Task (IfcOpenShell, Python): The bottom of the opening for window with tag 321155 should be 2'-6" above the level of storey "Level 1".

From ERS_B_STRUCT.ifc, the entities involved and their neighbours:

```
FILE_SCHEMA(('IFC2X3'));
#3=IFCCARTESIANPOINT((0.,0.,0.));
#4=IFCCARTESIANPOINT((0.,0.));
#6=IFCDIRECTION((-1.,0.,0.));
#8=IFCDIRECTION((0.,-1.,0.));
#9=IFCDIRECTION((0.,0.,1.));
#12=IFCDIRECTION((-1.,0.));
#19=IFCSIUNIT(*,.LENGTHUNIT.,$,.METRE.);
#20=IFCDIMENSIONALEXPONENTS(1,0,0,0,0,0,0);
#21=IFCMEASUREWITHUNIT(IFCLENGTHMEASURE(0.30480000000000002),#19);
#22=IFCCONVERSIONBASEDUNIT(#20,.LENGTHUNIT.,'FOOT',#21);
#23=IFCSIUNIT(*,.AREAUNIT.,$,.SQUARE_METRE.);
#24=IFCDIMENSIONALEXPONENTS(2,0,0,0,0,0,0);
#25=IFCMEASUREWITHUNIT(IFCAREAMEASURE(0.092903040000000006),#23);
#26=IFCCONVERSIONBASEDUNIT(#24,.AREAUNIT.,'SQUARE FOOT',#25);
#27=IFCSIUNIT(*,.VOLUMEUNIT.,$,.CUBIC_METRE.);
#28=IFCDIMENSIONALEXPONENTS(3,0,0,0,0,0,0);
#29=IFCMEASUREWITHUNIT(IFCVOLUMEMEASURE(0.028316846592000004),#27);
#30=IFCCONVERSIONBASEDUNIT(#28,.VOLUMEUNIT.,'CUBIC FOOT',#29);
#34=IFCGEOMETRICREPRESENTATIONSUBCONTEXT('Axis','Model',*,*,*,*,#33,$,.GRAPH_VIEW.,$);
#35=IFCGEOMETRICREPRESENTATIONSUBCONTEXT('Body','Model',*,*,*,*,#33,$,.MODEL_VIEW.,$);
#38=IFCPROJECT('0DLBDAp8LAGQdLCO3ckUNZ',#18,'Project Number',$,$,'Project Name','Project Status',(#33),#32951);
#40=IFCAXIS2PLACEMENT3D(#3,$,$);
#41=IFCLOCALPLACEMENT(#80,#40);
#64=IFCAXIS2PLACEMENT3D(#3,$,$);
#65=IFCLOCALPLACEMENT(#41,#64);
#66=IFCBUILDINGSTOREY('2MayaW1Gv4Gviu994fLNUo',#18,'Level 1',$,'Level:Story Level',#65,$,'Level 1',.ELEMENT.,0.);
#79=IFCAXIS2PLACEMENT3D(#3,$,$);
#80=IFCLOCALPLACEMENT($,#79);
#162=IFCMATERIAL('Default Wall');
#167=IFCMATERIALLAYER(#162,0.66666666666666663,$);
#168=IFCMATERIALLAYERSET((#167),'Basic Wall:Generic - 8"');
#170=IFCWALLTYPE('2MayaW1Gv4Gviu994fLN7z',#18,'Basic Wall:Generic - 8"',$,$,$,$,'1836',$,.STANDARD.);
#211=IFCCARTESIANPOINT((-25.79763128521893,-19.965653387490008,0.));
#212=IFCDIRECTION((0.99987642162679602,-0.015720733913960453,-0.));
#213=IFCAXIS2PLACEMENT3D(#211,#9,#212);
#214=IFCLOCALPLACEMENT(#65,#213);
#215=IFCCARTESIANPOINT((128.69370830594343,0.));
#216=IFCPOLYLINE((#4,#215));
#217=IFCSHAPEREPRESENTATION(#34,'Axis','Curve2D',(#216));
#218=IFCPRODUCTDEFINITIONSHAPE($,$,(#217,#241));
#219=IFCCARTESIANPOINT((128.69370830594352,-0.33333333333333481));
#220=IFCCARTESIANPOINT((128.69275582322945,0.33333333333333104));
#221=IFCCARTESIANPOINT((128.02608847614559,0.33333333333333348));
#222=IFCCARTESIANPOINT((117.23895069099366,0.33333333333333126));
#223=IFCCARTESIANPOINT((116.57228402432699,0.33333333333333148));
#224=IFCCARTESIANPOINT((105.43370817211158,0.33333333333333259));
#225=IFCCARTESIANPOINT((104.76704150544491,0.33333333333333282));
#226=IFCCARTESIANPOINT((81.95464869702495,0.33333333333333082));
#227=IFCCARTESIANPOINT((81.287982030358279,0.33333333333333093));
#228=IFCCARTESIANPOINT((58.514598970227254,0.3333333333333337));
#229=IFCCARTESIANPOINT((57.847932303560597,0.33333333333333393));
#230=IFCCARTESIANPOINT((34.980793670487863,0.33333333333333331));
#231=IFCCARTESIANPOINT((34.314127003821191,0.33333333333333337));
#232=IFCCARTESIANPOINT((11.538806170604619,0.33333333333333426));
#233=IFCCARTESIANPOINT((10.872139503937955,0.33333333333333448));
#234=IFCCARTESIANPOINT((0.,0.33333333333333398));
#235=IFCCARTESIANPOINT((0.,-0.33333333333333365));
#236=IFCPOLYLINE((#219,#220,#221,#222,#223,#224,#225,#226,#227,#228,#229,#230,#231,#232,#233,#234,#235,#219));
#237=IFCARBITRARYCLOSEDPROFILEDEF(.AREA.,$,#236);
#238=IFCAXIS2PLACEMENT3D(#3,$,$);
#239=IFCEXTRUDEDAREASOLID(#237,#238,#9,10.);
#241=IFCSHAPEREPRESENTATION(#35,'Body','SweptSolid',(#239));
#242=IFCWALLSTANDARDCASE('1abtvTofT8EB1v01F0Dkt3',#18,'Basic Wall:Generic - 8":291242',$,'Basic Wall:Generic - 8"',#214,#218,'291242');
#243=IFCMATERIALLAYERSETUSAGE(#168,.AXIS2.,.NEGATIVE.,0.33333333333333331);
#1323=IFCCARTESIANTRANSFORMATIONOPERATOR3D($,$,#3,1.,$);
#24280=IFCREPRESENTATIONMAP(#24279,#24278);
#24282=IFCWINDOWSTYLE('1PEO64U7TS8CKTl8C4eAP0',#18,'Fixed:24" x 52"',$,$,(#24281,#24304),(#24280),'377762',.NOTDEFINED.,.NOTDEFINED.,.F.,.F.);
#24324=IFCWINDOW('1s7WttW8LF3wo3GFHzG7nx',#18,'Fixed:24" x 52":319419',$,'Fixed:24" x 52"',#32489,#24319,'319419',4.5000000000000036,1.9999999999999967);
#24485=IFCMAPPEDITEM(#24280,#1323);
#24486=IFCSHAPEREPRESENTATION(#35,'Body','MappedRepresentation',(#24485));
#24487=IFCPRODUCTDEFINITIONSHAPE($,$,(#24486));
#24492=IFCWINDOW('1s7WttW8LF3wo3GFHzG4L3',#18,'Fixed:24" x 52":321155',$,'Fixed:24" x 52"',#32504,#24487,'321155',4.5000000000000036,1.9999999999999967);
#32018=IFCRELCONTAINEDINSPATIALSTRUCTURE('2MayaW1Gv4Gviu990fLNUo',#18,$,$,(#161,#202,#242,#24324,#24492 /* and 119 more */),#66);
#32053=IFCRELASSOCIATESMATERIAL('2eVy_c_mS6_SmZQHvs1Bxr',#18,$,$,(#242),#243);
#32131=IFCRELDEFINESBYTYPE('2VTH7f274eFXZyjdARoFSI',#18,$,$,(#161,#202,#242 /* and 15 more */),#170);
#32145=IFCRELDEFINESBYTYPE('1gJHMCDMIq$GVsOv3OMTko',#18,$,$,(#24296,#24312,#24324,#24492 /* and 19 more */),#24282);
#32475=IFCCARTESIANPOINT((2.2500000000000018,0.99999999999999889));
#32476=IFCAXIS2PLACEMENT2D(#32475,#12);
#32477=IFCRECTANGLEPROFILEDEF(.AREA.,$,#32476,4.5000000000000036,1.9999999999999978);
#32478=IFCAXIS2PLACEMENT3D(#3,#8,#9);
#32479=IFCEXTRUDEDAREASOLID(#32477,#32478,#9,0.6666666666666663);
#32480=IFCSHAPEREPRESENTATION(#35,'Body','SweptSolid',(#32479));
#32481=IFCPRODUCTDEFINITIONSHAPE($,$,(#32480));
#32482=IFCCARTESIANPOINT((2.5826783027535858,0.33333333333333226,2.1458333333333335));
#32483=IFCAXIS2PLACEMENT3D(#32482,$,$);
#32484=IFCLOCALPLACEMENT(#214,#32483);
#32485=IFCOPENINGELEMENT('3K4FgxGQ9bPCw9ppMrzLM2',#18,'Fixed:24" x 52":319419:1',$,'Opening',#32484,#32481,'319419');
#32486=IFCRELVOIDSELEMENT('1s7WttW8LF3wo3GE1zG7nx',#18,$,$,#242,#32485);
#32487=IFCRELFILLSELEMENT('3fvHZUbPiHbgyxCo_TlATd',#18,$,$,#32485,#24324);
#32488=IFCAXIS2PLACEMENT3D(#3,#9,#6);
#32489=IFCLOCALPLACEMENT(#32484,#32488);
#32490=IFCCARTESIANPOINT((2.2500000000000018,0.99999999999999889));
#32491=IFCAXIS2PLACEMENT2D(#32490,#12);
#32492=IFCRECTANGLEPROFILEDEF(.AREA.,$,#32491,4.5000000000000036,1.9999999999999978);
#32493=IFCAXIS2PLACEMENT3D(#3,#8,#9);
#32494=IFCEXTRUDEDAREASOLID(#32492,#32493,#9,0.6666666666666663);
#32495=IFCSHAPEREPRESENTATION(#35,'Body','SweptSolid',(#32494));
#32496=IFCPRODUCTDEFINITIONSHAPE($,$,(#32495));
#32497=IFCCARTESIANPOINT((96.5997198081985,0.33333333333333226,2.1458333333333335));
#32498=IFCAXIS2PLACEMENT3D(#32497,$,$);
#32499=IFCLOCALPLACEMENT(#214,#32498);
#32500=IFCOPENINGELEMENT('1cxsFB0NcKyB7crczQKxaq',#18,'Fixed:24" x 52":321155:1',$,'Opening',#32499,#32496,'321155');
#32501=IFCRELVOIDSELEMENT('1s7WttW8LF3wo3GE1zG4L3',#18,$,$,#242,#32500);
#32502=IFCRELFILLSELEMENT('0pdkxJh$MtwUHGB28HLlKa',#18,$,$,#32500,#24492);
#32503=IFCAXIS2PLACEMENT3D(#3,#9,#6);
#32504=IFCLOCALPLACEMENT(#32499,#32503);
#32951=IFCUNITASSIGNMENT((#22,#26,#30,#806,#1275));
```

```python
import numpy as np
import ifcopenshell
import ifcopenshell.api.geometry
import ifcopenshell.geom
import ifcopenshell.util.element
import ifcopenshell.util.placement
import ifcopenshell.util.shape
import ifcopenshell.util.unit

model = ifcopenshell.open("ERS_B_STRUCT.ifc")
unit_scale = ifcopenshell.util.unit.calculate_unit_scale(model)

window = model.by_guid("1s7WttW8LF3wo3GFHzG4L3")
opening = window.FillsVoids[0].RelatingOpeningElement
storey = ifcopenshell.util.element.get_container(window, ifc_class="IfcBuildingStorey")
level = ifcopenshell.util.placement.get_local_placement(storey.ObjectPlacement)[2, 3]

# The opening's origin need not be at the sill, so measure its lowest point.
shape = ifcopenshell.geom.create_shape(ifcopenshell.geom.settings(), opening)
bottom = ifcopenshell.util.shape.get_shape_bottom_elevation(shape, shape.geometry) / unit_scale
dz = level + 30 * 0.0254 / unit_scale - bottom

shift = np.array([0.0, 0.0, dz])
# The window is placed relative to its opening, so it follows when the opening moves.
matrix = ifcopenshell.util.placement.get_local_placement(opening.ObjectPlacement)
matrix[:3, 3] += shift
ifcopenshell.api.geometry.edit_object_placement(
    model, product=opening, matrix=matrix, is_si=False, should_transform_children=True
)

print(f"moved by {dz * unit_scale:+.3f} m")

model.write("ERS_B_STRUCT_updated.ifc")
```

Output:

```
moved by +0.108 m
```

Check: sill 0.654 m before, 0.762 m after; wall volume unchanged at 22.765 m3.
